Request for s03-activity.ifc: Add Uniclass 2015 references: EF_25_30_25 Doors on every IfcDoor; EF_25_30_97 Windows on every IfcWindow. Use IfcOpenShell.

First a look at what the model holds.

```python
import ifcopenshell

model = ifcopenshell.open("s03-activity.ifc")
print(model.schema)
print("classifications:", [c.Name for c in model.by_type("IfcClassification")])
for ifc_class in ("IfcDoor", "IfcRoof", "IfcStair", "IfcWall", "IfcWindow"):
    print(ifc_class, len(model.by_type(ifc_class)))
```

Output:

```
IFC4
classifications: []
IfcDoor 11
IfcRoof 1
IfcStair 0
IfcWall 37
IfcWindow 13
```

```python
import ifcopenshell
import ifcopenshell.api.classification

model = ifcopenshell.open("s03-activity.ifc")

system = ifcopenshell.api.classification.add_classification(model, classification="Uniclass 2015")

codes = {
    "IfcDoor": ("EF_25_30_25", "Doors"),
    "IfcWindow": ("EF_25_30_97", "Windows"),
}
for ifc_class, (code, name) in codes.items():
    products = model.by_type(ifc_class)
    ifcopenshell.api.classification.add_reference(
        model, products=products, classification=system, identification=code, name=name
    )
    print(code, len(products))

model.write("s03-activity_edited.ifc")
```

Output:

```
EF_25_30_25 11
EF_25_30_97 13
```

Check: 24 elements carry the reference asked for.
